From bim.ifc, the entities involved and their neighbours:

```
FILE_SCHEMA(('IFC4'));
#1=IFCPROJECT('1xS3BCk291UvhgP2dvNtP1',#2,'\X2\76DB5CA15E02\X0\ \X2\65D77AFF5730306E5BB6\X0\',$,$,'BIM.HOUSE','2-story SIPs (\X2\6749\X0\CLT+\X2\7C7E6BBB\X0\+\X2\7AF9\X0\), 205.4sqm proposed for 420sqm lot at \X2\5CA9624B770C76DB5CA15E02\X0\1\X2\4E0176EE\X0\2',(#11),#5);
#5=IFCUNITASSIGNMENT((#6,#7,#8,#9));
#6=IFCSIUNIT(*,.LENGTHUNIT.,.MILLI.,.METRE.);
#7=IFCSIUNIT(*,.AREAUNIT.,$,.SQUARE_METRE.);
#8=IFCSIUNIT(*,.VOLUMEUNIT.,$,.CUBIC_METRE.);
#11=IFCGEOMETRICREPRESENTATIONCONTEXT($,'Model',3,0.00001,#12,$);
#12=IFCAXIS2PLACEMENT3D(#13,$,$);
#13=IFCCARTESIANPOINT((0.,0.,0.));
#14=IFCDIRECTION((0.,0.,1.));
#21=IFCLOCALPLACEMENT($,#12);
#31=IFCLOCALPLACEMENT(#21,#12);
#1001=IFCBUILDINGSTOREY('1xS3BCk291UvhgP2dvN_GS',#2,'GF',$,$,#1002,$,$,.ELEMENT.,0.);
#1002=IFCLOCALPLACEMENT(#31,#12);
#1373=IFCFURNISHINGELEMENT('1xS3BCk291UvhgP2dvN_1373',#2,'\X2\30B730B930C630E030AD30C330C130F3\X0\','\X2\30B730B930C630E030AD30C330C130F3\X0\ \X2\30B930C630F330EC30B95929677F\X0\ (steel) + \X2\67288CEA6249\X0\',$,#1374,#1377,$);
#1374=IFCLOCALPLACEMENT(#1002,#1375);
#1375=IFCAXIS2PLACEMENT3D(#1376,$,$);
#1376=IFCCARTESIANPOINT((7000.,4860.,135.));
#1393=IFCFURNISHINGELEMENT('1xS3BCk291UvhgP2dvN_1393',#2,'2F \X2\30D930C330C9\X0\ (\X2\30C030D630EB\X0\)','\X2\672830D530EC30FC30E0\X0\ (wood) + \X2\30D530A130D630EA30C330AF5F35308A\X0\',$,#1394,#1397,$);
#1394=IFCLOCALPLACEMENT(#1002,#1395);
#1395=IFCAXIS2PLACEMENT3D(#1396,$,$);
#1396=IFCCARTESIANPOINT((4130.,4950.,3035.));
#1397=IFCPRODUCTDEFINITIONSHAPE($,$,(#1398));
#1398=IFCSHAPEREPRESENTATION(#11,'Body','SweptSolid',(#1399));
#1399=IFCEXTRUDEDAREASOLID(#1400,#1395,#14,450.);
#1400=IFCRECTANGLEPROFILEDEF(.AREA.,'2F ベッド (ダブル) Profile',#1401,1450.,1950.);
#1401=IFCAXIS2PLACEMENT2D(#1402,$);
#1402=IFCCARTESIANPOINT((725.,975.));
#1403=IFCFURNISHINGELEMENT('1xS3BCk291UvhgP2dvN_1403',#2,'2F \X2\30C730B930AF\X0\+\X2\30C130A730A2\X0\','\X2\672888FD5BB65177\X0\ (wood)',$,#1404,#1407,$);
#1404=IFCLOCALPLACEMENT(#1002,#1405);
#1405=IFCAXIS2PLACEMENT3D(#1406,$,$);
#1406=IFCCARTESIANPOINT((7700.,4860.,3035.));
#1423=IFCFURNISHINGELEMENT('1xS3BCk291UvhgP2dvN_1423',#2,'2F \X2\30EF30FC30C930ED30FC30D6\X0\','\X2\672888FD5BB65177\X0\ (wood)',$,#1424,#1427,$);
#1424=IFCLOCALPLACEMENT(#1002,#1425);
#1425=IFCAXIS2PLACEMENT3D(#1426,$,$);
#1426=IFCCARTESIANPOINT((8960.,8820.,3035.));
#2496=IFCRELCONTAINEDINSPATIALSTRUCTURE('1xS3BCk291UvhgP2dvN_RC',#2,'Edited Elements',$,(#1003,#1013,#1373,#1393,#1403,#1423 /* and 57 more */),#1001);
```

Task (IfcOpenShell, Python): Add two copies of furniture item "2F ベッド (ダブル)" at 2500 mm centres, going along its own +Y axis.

```python
import ifcopenshell
import ifcopenshell.api.geometry
import ifcopenshell.api.root
import ifcopenshell.util.element
import ifcopenshell.util.placement
import ifcopenshell.util.unit

model = ifcopenshell.open("bim.ifc")
unit_scale = ifcopenshell.util.unit.calculate_unit_scale(model)


def reuse_history(source, copy):
    """copy_class also copies each property set's owner history, people and application; keep the originals."""
    for rel in copy.IsDefinedBy:
        if rel.is_a("IfcRelDefinesByProperties") and (history := rel.RelatingPropertyDefinition.OwnerHistory):
            rel.RelatingPropertyDefinition.OwnerHistory = source.OwnerHistory
            ifcopenshell.util.element.remove_deep2(model, history)


source = model.by_id(1393)
base = ifcopenshell.util.placement.get_local_placement(source.ObjectPlacement)
step = base[:3, 1] * 2.5 / unit_scale

for i in range(1, 3):
    copy = ifcopenshell.api.root.copy_class(model, product=source)
    copy.Representation = ifcopenshell.util.element.copy_deep(
        model, source.Representation, exclude=["IfcGeometricRepresentationContext", "IfcRepresentationMap"]
    )
    reuse_history(source, copy)
    matrix = base.copy()
    matrix[:3, 3] += i * step
    print("added at", matrix[:3, 3].round(3) + 0.0)
    ifcopenshell.api.geometry.edit_object_placement(model, product=copy, matrix=matrix, is_si=False)

model.write("bim_updated.ifc")
```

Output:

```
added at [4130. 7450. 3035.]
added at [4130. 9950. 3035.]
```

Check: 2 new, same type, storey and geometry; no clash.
